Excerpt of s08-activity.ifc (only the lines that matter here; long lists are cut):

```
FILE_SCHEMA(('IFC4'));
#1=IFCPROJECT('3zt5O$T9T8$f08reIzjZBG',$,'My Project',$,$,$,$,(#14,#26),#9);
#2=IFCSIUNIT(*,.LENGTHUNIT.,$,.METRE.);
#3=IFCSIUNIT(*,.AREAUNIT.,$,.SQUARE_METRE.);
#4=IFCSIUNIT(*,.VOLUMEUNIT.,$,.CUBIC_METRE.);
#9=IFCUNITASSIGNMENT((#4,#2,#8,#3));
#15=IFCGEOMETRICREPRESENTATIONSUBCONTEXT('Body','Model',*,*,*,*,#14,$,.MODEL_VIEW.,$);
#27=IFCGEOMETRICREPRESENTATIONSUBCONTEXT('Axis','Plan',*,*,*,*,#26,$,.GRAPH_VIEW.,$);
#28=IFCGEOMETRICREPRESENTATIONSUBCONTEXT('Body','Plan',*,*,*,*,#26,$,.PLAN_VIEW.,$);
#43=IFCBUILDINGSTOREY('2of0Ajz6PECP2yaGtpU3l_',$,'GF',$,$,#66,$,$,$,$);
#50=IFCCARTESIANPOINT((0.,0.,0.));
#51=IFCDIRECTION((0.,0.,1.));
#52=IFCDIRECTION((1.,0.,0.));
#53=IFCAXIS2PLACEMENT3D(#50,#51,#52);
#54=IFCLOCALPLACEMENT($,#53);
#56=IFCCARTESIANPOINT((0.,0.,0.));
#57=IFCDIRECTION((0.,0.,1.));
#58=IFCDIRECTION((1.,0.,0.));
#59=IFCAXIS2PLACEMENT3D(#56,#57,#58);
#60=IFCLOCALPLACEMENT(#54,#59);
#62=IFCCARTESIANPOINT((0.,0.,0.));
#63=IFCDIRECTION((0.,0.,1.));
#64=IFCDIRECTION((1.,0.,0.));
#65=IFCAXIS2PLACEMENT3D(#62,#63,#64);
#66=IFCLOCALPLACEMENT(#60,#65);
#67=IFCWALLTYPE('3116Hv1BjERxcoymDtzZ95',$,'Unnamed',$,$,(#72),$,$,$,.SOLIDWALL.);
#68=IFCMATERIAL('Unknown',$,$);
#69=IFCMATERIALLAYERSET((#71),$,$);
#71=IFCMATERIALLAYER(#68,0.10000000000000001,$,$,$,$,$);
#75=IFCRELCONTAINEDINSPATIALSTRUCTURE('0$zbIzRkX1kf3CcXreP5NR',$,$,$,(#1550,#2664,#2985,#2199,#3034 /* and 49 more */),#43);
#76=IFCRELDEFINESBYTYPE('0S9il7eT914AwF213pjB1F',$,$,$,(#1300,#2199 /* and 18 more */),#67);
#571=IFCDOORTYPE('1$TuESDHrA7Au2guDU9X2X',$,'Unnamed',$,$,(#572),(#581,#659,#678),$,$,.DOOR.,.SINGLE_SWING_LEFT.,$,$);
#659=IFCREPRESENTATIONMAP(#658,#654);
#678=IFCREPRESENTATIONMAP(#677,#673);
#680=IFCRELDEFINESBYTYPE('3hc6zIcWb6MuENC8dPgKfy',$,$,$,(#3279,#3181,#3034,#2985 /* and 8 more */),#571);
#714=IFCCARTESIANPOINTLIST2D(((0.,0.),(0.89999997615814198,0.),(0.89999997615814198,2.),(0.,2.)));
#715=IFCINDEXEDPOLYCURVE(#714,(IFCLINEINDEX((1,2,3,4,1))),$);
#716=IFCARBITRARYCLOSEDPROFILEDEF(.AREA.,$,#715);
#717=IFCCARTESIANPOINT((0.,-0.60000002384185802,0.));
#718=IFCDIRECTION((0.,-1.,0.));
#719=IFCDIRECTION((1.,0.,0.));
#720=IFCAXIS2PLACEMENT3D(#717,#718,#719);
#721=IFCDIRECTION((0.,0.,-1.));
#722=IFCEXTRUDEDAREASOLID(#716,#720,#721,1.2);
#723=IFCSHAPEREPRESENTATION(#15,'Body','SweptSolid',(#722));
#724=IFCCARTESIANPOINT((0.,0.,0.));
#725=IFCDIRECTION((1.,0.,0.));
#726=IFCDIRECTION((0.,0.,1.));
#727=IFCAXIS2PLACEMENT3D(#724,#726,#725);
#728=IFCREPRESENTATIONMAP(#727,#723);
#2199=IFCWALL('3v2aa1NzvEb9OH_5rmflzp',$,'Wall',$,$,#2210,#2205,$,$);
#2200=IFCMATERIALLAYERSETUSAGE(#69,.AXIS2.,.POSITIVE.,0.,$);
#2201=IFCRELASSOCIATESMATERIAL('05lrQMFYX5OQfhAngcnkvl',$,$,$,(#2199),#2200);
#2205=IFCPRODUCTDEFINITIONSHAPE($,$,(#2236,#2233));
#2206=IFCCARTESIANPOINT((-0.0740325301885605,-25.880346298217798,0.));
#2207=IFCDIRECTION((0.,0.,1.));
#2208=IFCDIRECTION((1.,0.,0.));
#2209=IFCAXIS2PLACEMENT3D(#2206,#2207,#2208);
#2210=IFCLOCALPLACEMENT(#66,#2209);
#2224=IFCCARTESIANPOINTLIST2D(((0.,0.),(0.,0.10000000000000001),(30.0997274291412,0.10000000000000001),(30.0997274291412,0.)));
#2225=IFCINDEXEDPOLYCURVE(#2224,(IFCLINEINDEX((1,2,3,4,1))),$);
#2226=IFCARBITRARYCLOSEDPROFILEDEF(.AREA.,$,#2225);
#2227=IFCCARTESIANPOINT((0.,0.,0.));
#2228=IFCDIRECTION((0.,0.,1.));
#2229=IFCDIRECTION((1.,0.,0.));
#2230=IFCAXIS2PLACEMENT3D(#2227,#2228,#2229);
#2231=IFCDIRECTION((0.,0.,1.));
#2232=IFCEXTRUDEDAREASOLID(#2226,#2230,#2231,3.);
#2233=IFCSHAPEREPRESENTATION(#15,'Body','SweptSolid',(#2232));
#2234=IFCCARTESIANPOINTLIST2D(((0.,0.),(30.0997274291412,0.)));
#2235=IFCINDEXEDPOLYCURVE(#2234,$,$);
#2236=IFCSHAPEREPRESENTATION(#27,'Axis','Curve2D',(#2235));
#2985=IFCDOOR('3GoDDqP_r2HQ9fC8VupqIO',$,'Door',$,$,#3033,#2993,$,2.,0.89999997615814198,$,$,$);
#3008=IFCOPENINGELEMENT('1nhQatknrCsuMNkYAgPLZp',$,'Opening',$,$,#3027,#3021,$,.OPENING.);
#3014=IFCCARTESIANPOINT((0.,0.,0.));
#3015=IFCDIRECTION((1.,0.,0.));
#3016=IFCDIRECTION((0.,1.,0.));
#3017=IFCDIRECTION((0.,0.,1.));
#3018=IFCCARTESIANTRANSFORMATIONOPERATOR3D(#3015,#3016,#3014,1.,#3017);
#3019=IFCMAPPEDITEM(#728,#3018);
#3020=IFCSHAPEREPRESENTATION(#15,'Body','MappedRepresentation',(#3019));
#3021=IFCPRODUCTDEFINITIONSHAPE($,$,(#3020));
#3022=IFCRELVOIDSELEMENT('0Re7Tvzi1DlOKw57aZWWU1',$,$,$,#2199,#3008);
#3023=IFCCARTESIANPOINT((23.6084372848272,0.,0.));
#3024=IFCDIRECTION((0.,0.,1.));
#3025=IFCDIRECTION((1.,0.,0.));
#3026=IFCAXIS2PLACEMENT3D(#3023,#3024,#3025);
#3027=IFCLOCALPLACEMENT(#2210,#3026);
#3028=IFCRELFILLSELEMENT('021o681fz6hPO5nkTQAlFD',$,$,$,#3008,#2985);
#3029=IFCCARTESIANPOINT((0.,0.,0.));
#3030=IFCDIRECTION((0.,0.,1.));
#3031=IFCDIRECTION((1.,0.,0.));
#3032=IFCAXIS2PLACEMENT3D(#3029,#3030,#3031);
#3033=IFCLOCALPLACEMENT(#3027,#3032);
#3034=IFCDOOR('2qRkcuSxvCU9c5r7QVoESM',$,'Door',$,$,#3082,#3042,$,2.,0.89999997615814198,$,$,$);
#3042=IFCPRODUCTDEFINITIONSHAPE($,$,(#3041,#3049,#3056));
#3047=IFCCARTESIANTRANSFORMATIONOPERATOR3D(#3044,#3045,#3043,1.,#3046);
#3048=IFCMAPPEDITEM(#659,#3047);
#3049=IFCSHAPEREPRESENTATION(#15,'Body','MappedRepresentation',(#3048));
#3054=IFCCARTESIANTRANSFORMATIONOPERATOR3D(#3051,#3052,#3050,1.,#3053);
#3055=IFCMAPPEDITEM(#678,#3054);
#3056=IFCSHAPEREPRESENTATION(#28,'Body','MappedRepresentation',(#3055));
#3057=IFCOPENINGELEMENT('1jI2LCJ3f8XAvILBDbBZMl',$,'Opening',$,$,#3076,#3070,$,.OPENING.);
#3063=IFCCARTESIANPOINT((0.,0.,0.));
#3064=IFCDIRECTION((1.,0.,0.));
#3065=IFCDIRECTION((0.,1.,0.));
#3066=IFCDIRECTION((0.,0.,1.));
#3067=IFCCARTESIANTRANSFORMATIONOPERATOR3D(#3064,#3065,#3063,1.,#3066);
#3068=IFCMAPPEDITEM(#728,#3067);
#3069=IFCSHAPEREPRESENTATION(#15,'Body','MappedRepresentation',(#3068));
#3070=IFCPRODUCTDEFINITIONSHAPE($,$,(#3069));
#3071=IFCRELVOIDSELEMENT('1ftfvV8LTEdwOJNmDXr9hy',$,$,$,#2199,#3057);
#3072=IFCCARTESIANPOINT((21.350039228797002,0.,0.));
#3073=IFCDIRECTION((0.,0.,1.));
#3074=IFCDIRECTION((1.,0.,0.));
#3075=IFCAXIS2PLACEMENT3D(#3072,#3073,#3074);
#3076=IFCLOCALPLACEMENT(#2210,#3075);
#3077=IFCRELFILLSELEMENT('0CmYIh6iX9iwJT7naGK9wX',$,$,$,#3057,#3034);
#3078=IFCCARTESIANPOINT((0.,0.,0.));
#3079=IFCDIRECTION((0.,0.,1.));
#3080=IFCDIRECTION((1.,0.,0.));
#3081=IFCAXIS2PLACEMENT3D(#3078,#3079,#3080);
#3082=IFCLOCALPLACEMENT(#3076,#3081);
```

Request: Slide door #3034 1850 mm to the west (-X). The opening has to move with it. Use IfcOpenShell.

```python
import ifcopenshell
import ifcopenshell.api.geometry
import ifcopenshell.util.placement
import ifcopenshell.util.unit

model = ifcopenshell.open("s08-activity.ifc")
unit_scale = ifcopenshell.util.unit.calculate_unit_scale(model)

door = model.by_guid("2qRkcuSxvCU9c5r7QVoESM")
opening = door.FillsVoids[0].RelatingOpeningElement
wall = opening.VoidsElements[0].RelatingBuildingElement

wall_matrix = ifcopenshell.util.placement.get_local_placement(wall.ObjectPlacement)
shift = wall_matrix[:3, 0] * -1.85 / unit_scale
before = ifcopenshell.util.placement.get_local_placement(door.ObjectPlacement)[:3, 3].copy()

# The door is placed relative to its opening, so it follows when the opening moves.
matrix = ifcopenshell.util.placement.get_local_placement(opening.ObjectPlacement)
matrix[:3, 3] += shift
ifcopenshell.api.geometry.edit_object_placement(
    model, product=opening, matrix=matrix, is_si=False, should_transform_children=True
)

after = ifcopenshell.util.placement.get_local_placement(door.ObjectPlacement)[:3, 3]
print("door moved by", (after - before).round(3) + 0.0)

model.write("s08-activity_rev.ifc")
```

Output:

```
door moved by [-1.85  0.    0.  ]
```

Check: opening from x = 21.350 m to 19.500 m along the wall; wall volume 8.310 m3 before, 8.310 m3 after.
